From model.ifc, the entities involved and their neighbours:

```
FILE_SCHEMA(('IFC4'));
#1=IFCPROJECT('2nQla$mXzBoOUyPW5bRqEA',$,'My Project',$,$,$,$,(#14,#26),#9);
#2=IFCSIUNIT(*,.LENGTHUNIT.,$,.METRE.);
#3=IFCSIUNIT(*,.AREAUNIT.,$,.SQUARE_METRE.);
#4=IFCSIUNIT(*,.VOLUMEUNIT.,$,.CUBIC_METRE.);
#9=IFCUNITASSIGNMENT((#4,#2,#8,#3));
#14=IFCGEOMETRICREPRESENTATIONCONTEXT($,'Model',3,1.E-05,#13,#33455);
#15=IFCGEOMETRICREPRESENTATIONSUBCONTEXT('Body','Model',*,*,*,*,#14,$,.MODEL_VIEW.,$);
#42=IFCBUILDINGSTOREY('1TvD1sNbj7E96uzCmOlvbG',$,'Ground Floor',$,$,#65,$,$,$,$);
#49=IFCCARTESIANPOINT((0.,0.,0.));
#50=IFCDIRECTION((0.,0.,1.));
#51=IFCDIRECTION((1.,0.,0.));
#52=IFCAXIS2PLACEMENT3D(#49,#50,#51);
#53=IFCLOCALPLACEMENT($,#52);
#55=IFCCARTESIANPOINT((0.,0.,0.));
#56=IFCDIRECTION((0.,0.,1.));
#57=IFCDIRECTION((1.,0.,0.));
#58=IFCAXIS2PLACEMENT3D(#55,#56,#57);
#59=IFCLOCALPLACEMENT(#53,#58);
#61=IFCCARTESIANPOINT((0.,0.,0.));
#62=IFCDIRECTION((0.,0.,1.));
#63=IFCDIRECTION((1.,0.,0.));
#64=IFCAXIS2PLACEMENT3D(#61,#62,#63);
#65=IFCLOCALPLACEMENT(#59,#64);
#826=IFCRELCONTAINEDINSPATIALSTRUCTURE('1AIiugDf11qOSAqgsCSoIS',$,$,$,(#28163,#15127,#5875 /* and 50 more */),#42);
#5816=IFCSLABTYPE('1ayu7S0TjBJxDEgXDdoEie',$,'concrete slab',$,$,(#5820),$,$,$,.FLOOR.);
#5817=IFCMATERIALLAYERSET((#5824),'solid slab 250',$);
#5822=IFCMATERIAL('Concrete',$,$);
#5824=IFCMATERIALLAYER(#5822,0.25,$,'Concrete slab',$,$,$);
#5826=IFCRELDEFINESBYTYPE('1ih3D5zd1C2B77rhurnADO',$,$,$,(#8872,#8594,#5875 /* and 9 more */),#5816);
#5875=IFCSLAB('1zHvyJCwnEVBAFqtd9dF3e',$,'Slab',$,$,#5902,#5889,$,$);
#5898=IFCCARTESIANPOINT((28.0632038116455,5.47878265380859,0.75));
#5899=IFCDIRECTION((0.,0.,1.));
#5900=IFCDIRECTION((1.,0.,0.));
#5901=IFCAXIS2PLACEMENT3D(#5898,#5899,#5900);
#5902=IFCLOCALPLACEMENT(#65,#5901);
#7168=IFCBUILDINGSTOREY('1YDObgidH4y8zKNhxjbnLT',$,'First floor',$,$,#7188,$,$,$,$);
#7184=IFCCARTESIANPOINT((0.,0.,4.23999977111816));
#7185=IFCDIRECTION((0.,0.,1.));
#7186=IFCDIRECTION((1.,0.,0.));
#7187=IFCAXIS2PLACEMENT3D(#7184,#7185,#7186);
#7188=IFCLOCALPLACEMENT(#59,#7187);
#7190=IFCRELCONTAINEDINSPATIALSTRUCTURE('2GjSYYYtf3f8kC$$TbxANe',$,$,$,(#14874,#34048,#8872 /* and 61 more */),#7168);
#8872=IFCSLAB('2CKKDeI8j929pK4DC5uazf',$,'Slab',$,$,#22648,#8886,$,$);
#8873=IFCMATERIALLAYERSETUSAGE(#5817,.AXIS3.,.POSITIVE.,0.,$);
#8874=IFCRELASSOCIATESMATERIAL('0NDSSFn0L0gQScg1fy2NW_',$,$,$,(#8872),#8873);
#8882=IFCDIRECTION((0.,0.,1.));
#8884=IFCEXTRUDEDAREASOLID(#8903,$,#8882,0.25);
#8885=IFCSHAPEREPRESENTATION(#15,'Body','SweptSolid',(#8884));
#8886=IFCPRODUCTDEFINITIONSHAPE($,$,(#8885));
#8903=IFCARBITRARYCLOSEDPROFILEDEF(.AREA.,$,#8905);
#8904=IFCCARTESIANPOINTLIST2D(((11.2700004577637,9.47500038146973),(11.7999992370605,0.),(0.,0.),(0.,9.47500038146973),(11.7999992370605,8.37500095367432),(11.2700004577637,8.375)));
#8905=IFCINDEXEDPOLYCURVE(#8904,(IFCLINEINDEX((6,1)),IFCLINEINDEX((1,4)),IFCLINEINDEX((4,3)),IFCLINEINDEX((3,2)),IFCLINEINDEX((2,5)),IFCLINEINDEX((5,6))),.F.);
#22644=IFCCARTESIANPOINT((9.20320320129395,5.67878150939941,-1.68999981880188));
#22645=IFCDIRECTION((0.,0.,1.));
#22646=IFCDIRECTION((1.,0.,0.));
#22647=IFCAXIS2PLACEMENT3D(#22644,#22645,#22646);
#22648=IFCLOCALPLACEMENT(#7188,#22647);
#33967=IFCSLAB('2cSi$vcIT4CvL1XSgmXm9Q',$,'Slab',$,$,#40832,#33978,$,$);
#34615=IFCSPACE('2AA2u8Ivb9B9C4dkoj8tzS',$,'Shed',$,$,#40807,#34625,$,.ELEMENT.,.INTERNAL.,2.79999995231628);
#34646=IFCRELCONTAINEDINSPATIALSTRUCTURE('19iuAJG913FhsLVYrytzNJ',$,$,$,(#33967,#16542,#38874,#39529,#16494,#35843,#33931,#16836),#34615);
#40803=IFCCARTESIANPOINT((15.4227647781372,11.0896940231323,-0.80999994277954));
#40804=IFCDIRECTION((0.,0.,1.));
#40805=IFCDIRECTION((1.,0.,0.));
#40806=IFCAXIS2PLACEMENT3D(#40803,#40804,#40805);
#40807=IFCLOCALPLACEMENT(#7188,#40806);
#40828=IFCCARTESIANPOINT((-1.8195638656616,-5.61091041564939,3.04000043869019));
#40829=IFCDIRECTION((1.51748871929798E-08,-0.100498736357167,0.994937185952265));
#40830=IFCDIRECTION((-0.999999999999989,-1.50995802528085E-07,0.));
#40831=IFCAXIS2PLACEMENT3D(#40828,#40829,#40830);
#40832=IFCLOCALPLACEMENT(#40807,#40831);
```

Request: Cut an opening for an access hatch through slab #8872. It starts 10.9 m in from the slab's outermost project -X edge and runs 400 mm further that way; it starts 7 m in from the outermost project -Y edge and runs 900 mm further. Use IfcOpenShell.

```python
import numpy as np
import ifcopenshell
import ifcopenshell.api.feature
import ifcopenshell.api.geometry
import ifcopenshell.api.root
import ifcopenshell.geom
import ifcopenshell.util.placement
import ifcopenshell.util.representation
import ifcopenshell.util.shape
import ifcopenshell.util.unit

model = ifcopenshell.open("model.ifc")
unit_scale = ifcopenshell.util.unit.calculate_unit_scale(model)
settings = ifcopenshell.geom.settings()


def volume(element):
    """Net volume in cubic metres, openings subtracted."""
    shape = ifcopenshell.geom.create_shape(settings, element)
    return ifcopenshell.util.shape.get_volume(shape.geometry)


slab = model.by_guid("2CKKDeI8j929pK4DC5uazf")
before = volume(slab)

# Extent in the slab's own axes, in metres. The edges named are its -X and -Y sides.
slab_shape = ifcopenshell.geom.create_shape(settings, slab)
vertices = ifcopenshell.util.shape.get_vertices(slab_shape.geometry)
x_min, y_min, bottom = vertices.min(axis=0)
top = vertices[:, 2].max()

opening = ifcopenshell.api.root.create_entity(model, ifc_class="IfcOpeningElement", name="Access hatch opening", predefined_type="OPENING")
context = ifcopenshell.util.representation.get_context(model, "Model", "Body", "MODEL_VIEW")
width, depth = 0.4, 0.9
outline = [(0.0, 0.0), (width, 0.0), (width, depth), (0.0, depth), (0.0, 0.0)]
# Overshoot both faces by 50 mm so the cut is clean.
shape = ifcopenshell.api.geometry.add_slab_representation(
    model, context=context, depth=top - bottom + 0.1, polyline=outline
)
ifcopenshell.api.geometry.assign_representation(model, product=opening, representation=shape)

matrix = ifcopenshell.util.placement.get_local_placement(slab.ObjectPlacement)
matrix[:, 3] = matrix @ np.append(np.array([x_min + 10.9, y_min + 7, bottom - 0.05]) / unit_scale, 1.0)
ifcopenshell.api.geometry.edit_object_placement(model, product=opening, matrix=matrix, is_si=False)
ifcopenshell.api.feature.add_feature(model, feature=opening, element=slab)

after = volume(slab)

print(f"slab volume {before:.3f} -> {after:.3f} m3")

model.write("model_edited.ifc")
```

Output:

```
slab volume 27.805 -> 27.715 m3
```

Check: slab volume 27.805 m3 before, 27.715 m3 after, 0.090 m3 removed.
